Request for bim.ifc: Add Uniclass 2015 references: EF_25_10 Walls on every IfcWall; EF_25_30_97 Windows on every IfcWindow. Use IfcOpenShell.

First a look at what the model holds.

```python
import ifcopenshell

model = ifcopenshell.open("bim.ifc")
print(model.schema)
print("classifications:", [c.Name for c in model.by_type("IfcClassification")])
for ifc_class in ("IfcDoor", "IfcRoof", "IfcStair", "IfcWall", "IfcWindow"):
    print(ifc_class, len(model.by_type(ifc_class)))
```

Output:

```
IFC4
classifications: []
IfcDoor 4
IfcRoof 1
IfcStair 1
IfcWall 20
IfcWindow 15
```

```python
import ifcopenshell
import ifcopenshell.api.classification

model = ifcopenshell.open("bim.ifc")

system = ifcopenshell.api.classification.add_classification(model, classification="Uniclass 2015")

codes = {
    "IfcWall": ("EF_25_10", "Walls"),
    "IfcWindow": ("EF_25_30_97", "Windows"),
}
for ifc_class, (code, name) in codes.items():
    products = model.by_type(ifc_class)
    ifcopenshell.api.classification.add_reference(
        model, products=products, classification=system, identification=code, name=name
    )
    print(code, len(products))

model.write("bim-out.ifc")
```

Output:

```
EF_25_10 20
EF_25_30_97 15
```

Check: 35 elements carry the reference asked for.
